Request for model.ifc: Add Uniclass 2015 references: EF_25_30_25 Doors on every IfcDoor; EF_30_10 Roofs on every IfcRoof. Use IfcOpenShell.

First a look at what the model holds.

```python
import ifcopenshell

model = ifcopenshell.open("model.ifc")
print(model.schema)
print("classifications:", [c.Name for c in model.by_type("IfcClassification")])
for ifc_class in ("IfcDoor", "IfcRoof", "IfcStair", "IfcWall", "IfcWindow"):
    print(ifc_class, len(model.by_type(ifc_class)))
```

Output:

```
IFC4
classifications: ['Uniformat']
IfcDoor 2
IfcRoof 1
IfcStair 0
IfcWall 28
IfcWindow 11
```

```python
import ifcopenshell
import ifcopenshell.api.classification

model = ifcopenshell.open("model.ifc")

system = ifcopenshell.api.classification.add_classification(model, classification="Uniclass 2015")

codes = {
    "IfcDoor": ("EF_25_30_25", "Doors"),
    "IfcRoof": ("EF_30_10", "Roofs"),
}
for ifc_class, (code, name) in codes.items():
    products = model.by_type(ifc_class)
    ifcopenshell.api.classification.add_reference(
        model, products=products, classification=system, identification=code, name=name
    )
    print(code, len(products))

model.write("model_v2.ifc")
```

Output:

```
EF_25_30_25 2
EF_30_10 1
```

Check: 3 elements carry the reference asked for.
